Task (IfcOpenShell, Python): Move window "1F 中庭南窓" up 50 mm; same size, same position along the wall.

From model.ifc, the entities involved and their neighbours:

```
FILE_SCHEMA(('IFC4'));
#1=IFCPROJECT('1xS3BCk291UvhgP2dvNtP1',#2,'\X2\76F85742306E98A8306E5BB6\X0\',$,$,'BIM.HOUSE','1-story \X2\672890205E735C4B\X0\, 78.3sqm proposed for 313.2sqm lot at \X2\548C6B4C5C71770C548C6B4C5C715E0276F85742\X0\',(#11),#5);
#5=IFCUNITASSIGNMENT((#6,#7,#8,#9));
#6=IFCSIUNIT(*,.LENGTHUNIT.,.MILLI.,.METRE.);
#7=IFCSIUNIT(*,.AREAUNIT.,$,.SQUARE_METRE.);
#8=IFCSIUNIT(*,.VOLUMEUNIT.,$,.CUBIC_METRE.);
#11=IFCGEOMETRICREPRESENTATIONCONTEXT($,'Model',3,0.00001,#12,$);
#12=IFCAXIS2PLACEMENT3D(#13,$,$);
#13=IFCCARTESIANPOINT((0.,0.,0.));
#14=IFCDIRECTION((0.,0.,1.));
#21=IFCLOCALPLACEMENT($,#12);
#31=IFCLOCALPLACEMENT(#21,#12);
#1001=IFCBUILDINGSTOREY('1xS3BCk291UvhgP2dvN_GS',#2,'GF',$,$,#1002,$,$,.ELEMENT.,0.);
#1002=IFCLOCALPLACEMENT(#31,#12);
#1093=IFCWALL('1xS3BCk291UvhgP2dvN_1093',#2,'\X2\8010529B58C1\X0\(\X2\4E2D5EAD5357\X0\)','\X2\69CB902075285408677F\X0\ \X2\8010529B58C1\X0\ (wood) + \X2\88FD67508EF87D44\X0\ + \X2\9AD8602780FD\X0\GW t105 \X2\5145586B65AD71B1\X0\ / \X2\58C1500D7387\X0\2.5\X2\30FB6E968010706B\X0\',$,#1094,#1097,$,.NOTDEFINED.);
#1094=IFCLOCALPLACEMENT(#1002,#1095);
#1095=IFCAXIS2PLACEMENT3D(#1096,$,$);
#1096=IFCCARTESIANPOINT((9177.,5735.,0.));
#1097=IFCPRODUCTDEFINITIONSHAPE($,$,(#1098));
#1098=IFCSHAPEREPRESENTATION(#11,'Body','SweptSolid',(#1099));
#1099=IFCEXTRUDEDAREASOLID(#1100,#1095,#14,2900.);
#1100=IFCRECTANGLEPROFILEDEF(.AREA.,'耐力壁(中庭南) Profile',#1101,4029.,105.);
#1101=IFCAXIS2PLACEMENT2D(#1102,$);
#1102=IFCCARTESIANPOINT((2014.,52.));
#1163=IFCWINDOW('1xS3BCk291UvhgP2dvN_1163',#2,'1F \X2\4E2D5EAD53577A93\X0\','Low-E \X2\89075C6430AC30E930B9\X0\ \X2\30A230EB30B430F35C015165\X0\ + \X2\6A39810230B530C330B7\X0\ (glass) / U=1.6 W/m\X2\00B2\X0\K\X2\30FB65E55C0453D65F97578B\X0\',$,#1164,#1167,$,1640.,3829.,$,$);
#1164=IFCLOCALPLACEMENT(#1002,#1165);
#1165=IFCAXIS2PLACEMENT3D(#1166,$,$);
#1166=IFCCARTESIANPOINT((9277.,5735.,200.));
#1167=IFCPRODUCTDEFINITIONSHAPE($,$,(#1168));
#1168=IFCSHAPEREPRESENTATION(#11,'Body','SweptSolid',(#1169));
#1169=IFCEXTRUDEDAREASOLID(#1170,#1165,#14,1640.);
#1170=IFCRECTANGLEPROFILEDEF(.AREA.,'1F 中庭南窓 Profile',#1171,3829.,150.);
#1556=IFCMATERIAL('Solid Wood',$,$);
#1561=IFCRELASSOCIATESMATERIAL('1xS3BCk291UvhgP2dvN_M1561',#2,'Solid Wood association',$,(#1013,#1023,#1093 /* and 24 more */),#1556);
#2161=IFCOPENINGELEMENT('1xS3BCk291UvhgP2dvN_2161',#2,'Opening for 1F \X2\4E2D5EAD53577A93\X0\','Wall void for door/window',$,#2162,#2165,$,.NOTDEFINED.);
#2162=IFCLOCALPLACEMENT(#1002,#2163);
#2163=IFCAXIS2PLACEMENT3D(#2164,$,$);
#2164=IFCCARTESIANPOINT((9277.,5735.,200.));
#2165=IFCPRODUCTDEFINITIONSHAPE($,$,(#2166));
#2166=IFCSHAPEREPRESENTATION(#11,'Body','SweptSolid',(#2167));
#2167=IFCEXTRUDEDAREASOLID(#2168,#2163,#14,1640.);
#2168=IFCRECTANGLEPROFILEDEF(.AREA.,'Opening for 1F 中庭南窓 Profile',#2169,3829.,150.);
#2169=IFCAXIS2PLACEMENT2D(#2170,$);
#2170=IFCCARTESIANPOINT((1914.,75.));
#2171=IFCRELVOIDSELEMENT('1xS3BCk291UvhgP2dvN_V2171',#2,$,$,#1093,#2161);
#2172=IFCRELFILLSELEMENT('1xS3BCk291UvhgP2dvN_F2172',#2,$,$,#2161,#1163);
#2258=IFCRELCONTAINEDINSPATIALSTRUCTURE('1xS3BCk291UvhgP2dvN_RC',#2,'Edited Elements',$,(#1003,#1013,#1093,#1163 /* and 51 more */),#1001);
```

```python
import numpy as np
import ifcopenshell
import ifcopenshell.api.geometry
import ifcopenshell.util.placement
import ifcopenshell.util.unit

model = ifcopenshell.open("model.ifc")
unit_scale = ifcopenshell.util.unit.calculate_unit_scale(model)

window = model.by_guid("1xS3BCk291UvhgP2dvN_1163")
opening = window.FillsVoids[0].RelatingOpeningElement
dz = 0.05 / unit_scale

shift = np.array([0.0, 0.0, dz])
# The window is not placed relative to its opening, so move both.
for product in (opening, window):
    matrix = ifcopenshell.util.placement.get_local_placement(product.ObjectPlacement)
    matrix[:3, 3] += shift
    ifcopenshell.api.geometry.edit_object_placement(model, product=product, matrix=matrix, is_si=False)

print(f"moved by {dz * unit_scale:+.3f} m")

model.write("model_updated.ifc")
```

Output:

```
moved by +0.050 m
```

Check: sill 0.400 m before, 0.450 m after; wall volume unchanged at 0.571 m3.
